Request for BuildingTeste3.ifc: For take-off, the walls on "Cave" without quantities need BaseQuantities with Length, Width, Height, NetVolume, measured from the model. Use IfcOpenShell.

First a look at what the model holds.

```python
import ifcopenshell
import ifcopenshell.util.element
import ifcopenshell.util.unit

model = ifcopenshell.open("BuildingTeste3.ifc")
print(model.schema)
for unit_type in ("LENGTHUNIT", "AREAUNIT", "VOLUMEUNIT"):
    print(unit_type, ifcopenshell.util.unit.calculate_unit_scale(model, unit_type))
storey = next(s for s in model.by_type("IfcBuildingStorey") if s.Name == "Cave")
walls = [e for e in ifcopenshell.util.element.get_decomposition(storey) if e.is_a("IfcWall")]
for e in sorted(walls, key=lambda e: e.id()):
    print(e.id(), e.is_a(), e.Name, list(ifcopenshell.util.element.get_psets(e, qtos_only=True)), sep=" | ")
```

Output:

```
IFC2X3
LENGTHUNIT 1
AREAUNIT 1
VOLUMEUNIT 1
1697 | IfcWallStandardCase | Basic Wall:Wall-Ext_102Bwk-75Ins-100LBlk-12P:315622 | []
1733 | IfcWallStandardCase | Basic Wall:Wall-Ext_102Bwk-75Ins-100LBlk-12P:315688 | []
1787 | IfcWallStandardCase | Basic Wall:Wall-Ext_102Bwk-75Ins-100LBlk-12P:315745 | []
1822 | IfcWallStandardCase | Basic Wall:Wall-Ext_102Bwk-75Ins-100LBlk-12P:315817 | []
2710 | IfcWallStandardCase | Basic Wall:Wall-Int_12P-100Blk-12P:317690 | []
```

```python
import ifcopenshell
import ifcopenshell.api.pset
import ifcopenshell.geom
import ifcopenshell.util.element
import ifcopenshell.util.shape
import ifcopenshell.util.unit

model = ifcopenshell.open("BuildingTeste3.ifc")
unit_scale = ifcopenshell.util.unit.calculate_unit_scale(model)
volume_scale = ifcopenshell.util.unit.calculate_unit_scale(model, "VOLUMEUNIT")
settings = ifcopenshell.geom.settings()

storey = next(s for s in model.by_type("IfcBuildingStorey") if s.Name == "Cave")
walls = [e for e in ifcopenshell.util.element.get_decomposition(storey) if e.is_a("IfcWall")]

for e in sorted(walls, key=lambda e: e.id()):
    if ifcopenshell.util.element.get_psets(e, qtos_only=True, should_inherit=False):
        continue
    # Geometry comes back in metres, in the element's own axes.
    shape = ifcopenshell.geom.create_shape(settings, e)
    values = {
        "Length": ifcopenshell.util.shape.get_x(shape.geometry) / unit_scale,
        "Width": ifcopenshell.util.shape.get_y(shape.geometry) / unit_scale,
        "Height": ifcopenshell.util.shape.get_z(shape.geometry) / unit_scale,
        "NetVolume": ifcopenshell.util.shape.get_volume(shape.geometry) / volume_scale,
    }
    qto = ifcopenshell.api.pset.add_qto(model, product=e, name="BaseQuantities")
    ifcopenshell.api.pset.edit_qto(model, qto=qto, properties=values)
    print(e.id(), {k: round(v, 3) for k, v in values.items()})

model.write("BuildingTeste3-out.ifc")
```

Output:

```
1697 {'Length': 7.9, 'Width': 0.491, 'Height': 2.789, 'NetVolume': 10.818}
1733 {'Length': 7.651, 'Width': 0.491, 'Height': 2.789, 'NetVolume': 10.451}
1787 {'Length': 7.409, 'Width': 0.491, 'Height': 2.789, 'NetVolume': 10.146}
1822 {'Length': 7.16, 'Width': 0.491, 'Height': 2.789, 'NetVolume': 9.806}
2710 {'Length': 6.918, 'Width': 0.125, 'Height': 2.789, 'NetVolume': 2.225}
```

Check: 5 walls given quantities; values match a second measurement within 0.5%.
